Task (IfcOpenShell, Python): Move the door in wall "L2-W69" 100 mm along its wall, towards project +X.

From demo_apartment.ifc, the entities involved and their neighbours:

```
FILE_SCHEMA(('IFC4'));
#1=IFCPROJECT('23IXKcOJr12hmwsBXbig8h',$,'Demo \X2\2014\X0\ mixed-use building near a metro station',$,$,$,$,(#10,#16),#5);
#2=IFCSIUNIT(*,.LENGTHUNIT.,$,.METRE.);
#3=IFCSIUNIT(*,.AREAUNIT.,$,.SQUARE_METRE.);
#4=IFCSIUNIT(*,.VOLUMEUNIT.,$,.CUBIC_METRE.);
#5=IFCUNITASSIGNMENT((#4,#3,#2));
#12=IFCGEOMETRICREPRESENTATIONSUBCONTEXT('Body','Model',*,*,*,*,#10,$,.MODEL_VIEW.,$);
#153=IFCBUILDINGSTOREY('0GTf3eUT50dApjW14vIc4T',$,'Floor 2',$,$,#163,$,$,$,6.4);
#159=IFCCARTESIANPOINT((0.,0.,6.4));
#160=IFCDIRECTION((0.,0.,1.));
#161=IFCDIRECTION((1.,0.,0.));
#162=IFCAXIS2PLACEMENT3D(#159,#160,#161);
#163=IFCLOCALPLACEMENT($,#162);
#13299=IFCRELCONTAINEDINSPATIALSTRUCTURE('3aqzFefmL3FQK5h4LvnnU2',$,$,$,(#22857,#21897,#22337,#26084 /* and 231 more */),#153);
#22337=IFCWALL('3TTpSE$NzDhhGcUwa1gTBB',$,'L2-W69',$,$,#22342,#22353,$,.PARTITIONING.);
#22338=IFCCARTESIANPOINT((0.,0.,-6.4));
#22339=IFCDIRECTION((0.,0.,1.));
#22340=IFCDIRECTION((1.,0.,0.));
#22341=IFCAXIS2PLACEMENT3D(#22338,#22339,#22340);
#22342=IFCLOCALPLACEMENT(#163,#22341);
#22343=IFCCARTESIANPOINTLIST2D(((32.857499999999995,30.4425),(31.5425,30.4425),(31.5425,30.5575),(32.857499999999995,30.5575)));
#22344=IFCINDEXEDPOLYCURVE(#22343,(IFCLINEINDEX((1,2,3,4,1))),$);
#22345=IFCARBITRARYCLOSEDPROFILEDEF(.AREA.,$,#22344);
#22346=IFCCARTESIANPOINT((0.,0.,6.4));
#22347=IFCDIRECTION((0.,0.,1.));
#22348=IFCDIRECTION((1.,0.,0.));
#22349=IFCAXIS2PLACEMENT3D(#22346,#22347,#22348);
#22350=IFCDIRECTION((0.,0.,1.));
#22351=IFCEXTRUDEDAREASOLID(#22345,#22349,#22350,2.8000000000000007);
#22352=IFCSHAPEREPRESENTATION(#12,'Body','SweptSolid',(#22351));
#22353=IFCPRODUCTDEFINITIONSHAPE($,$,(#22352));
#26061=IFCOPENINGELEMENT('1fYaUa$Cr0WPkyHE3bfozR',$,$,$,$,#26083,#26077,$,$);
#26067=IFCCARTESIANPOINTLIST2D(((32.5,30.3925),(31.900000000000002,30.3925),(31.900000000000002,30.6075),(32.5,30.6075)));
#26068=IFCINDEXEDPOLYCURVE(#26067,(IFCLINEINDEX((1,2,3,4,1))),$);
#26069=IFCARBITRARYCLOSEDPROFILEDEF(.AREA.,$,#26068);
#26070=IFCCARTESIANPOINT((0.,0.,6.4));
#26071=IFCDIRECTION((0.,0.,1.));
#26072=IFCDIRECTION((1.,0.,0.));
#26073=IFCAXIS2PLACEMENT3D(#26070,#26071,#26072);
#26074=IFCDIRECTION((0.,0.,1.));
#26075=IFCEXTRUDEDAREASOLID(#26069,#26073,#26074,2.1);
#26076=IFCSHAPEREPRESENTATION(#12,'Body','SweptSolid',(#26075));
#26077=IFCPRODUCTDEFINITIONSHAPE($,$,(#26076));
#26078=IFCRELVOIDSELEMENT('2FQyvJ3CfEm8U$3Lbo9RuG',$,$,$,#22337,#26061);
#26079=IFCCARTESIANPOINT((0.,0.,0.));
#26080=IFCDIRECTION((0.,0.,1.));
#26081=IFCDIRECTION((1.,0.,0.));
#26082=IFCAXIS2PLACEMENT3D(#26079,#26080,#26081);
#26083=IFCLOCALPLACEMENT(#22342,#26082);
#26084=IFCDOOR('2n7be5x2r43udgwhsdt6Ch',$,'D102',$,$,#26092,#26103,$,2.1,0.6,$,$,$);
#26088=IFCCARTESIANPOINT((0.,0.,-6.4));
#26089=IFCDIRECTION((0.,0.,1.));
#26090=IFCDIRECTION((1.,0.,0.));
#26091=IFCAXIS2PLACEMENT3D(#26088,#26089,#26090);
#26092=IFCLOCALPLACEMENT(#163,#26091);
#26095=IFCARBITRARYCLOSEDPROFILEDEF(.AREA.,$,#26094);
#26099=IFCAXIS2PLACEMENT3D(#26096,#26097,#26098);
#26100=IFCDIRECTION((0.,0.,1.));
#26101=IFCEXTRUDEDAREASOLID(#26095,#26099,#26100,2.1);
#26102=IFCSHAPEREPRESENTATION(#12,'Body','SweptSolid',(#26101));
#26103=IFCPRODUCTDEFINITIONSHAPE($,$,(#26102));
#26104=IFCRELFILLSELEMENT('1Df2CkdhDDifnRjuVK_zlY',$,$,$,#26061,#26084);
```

```python
import ifcopenshell
import ifcopenshell.api.geometry
import ifcopenshell.util.placement
import ifcopenshell.util.unit

model = ifcopenshell.open("demo_apartment.ifc")
unit_scale = ifcopenshell.util.unit.calculate_unit_scale(model)

door = model.by_id(26084)
opening = door.FillsVoids[0].RelatingOpeningElement
wall = opening.VoidsElements[0].RelatingBuildingElement

wall_matrix = ifcopenshell.util.placement.get_local_placement(wall.ObjectPlacement)
shift = wall_matrix[:3, 0] * 0.1 / unit_scale
before = ifcopenshell.util.placement.get_local_placement(door.ObjectPlacement)[:3, 3].copy()

# The door is not placed relative to its opening, so move both.
for product in (opening, door):
    matrix = ifcopenshell.util.placement.get_local_placement(product.ObjectPlacement)
    matrix[:3, 3] += shift
    ifcopenshell.api.geometry.edit_object_placement(model, product=product, matrix=matrix, is_si=False)

after = ifcopenshell.util.placement.get_local_placement(door.ObjectPlacement)[:3, 3]
print("door moved by", (after - before).round(3) + 0.0)

model.write("demo_apartment_edited.ifc")
```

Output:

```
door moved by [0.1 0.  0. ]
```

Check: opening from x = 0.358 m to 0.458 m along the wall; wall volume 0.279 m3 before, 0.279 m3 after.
